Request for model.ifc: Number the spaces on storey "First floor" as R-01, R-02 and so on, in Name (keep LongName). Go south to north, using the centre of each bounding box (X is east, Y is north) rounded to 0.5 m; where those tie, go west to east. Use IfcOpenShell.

First a look at what the model holds.

```python
import ifcopenshell
import ifcopenshell.util.element
import ifcopenshell.util.placement

model = ifcopenshell.open("model.ifc")
print(model.schema)
storey = next(s for s in model.by_type("IfcBuildingStorey") if s.Name == "First floor")
spaces = [e for e in ifcopenshell.util.element.get_decomposition(storey) if e.is_a("IfcSpace")]
for e in sorted(spaces, key=lambda e: e.id()):
    origin = ifcopenshell.util.placement.get_local_placement(e.ObjectPlacement)[:3, 3]
    print(e.id(), e.Name, e.LongName, origin.round(2) + 0.0, sep=" | ")
```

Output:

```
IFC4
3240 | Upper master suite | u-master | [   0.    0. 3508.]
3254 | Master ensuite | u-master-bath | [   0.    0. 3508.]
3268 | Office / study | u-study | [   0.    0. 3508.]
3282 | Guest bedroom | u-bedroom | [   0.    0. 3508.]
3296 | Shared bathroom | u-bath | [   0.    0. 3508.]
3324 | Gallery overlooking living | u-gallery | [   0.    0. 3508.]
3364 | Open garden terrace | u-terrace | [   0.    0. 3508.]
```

```python
import ifcopenshell
import ifcopenshell.geom
import ifcopenshell.util.element
import ifcopenshell.util.shape

model = ifcopenshell.open("model.ifc")
settings = ifcopenshell.geom.settings()
settings.set("use-world-coords", True)


def centre(element):
    shape = ifcopenshell.geom.create_shape(settings, element)
    return ifcopenshell.util.shape.get_bbox_centroid(shape.geometry)


storey = next(s for s in model.by_type("IfcBuildingStorey") if s.Name == "First floor")
spaces = [e for e in ifcopenshell.util.element.get_decomposition(storey) if e.is_a("IfcSpace")]

# Insertion points can sit at a corner or the storey origin, so sort by the geometry (in metres).
centres = {e: centre(e) for e in spaces}
spaces.sort(key=lambda e: (round(centres[e][1] / 0.5), centres[e][0]))

for i, e in enumerate(spaces, start=1):
    number = f"R-{i:02d}"
    e.Name = number
    print(e.id(), number)

model.write("model-out.ifc")
```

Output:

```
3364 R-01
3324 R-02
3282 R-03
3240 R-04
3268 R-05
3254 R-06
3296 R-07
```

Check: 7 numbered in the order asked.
